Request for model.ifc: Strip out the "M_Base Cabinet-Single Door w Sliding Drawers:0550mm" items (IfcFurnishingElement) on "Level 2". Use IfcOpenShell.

First a look at what the model holds.

```python
import ifcopenshell
import ifcopenshell.util.element

model = ifcopenshell.open("model.ifc")
print(model.schema)
storey = next(s for s in model.by_type("IfcBuildingStorey") if s.Name == "Level 2")
furniture = [e for e in ifcopenshell.util.element.get_decomposition(storey) if e.is_a("IfcFurnishingElement")]
seen = {}
for e in furniture:
    element_type = ifcopenshell.util.element.get_type(e)
    name = element_type.Name if element_type not in (None, e) else None
    seen[name] = seen.get(name, 0) + 1
for name, count in sorted(seen.items(), key=str):
    print(count, "x", name)
```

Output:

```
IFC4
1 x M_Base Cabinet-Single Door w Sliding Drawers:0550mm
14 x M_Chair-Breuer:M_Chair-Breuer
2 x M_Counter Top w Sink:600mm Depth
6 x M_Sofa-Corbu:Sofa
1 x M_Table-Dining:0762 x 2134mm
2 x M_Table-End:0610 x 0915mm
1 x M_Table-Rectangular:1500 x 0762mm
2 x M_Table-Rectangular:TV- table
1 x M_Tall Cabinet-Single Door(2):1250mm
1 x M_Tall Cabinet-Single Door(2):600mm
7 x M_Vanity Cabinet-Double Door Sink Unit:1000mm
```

```python
import ifcopenshell
import ifcopenshell.api.root
import ifcopenshell.util.element

model = ifcopenshell.open("model.ifc")

storey = next(s for s in model.by_type("IfcBuildingStorey") if s.Name == "Level 2")
furniture = [e for e in ifcopenshell.util.element.get_decomposition(storey) if e.is_a("IfcFurnishingElement")]
targets = [e for e in furniture if (t := ifcopenshell.util.element.get_type(e)) not in (None, e) and t.Name == "M_Base Cabinet-Single Door w Sliding Drawers:0550mm"]

for e in targets:
    ifcopenshell.api.root.remove_product(model, product=e)
print(len(targets), "removed")

model.write("model_edited.ifc")
```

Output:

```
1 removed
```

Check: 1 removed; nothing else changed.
